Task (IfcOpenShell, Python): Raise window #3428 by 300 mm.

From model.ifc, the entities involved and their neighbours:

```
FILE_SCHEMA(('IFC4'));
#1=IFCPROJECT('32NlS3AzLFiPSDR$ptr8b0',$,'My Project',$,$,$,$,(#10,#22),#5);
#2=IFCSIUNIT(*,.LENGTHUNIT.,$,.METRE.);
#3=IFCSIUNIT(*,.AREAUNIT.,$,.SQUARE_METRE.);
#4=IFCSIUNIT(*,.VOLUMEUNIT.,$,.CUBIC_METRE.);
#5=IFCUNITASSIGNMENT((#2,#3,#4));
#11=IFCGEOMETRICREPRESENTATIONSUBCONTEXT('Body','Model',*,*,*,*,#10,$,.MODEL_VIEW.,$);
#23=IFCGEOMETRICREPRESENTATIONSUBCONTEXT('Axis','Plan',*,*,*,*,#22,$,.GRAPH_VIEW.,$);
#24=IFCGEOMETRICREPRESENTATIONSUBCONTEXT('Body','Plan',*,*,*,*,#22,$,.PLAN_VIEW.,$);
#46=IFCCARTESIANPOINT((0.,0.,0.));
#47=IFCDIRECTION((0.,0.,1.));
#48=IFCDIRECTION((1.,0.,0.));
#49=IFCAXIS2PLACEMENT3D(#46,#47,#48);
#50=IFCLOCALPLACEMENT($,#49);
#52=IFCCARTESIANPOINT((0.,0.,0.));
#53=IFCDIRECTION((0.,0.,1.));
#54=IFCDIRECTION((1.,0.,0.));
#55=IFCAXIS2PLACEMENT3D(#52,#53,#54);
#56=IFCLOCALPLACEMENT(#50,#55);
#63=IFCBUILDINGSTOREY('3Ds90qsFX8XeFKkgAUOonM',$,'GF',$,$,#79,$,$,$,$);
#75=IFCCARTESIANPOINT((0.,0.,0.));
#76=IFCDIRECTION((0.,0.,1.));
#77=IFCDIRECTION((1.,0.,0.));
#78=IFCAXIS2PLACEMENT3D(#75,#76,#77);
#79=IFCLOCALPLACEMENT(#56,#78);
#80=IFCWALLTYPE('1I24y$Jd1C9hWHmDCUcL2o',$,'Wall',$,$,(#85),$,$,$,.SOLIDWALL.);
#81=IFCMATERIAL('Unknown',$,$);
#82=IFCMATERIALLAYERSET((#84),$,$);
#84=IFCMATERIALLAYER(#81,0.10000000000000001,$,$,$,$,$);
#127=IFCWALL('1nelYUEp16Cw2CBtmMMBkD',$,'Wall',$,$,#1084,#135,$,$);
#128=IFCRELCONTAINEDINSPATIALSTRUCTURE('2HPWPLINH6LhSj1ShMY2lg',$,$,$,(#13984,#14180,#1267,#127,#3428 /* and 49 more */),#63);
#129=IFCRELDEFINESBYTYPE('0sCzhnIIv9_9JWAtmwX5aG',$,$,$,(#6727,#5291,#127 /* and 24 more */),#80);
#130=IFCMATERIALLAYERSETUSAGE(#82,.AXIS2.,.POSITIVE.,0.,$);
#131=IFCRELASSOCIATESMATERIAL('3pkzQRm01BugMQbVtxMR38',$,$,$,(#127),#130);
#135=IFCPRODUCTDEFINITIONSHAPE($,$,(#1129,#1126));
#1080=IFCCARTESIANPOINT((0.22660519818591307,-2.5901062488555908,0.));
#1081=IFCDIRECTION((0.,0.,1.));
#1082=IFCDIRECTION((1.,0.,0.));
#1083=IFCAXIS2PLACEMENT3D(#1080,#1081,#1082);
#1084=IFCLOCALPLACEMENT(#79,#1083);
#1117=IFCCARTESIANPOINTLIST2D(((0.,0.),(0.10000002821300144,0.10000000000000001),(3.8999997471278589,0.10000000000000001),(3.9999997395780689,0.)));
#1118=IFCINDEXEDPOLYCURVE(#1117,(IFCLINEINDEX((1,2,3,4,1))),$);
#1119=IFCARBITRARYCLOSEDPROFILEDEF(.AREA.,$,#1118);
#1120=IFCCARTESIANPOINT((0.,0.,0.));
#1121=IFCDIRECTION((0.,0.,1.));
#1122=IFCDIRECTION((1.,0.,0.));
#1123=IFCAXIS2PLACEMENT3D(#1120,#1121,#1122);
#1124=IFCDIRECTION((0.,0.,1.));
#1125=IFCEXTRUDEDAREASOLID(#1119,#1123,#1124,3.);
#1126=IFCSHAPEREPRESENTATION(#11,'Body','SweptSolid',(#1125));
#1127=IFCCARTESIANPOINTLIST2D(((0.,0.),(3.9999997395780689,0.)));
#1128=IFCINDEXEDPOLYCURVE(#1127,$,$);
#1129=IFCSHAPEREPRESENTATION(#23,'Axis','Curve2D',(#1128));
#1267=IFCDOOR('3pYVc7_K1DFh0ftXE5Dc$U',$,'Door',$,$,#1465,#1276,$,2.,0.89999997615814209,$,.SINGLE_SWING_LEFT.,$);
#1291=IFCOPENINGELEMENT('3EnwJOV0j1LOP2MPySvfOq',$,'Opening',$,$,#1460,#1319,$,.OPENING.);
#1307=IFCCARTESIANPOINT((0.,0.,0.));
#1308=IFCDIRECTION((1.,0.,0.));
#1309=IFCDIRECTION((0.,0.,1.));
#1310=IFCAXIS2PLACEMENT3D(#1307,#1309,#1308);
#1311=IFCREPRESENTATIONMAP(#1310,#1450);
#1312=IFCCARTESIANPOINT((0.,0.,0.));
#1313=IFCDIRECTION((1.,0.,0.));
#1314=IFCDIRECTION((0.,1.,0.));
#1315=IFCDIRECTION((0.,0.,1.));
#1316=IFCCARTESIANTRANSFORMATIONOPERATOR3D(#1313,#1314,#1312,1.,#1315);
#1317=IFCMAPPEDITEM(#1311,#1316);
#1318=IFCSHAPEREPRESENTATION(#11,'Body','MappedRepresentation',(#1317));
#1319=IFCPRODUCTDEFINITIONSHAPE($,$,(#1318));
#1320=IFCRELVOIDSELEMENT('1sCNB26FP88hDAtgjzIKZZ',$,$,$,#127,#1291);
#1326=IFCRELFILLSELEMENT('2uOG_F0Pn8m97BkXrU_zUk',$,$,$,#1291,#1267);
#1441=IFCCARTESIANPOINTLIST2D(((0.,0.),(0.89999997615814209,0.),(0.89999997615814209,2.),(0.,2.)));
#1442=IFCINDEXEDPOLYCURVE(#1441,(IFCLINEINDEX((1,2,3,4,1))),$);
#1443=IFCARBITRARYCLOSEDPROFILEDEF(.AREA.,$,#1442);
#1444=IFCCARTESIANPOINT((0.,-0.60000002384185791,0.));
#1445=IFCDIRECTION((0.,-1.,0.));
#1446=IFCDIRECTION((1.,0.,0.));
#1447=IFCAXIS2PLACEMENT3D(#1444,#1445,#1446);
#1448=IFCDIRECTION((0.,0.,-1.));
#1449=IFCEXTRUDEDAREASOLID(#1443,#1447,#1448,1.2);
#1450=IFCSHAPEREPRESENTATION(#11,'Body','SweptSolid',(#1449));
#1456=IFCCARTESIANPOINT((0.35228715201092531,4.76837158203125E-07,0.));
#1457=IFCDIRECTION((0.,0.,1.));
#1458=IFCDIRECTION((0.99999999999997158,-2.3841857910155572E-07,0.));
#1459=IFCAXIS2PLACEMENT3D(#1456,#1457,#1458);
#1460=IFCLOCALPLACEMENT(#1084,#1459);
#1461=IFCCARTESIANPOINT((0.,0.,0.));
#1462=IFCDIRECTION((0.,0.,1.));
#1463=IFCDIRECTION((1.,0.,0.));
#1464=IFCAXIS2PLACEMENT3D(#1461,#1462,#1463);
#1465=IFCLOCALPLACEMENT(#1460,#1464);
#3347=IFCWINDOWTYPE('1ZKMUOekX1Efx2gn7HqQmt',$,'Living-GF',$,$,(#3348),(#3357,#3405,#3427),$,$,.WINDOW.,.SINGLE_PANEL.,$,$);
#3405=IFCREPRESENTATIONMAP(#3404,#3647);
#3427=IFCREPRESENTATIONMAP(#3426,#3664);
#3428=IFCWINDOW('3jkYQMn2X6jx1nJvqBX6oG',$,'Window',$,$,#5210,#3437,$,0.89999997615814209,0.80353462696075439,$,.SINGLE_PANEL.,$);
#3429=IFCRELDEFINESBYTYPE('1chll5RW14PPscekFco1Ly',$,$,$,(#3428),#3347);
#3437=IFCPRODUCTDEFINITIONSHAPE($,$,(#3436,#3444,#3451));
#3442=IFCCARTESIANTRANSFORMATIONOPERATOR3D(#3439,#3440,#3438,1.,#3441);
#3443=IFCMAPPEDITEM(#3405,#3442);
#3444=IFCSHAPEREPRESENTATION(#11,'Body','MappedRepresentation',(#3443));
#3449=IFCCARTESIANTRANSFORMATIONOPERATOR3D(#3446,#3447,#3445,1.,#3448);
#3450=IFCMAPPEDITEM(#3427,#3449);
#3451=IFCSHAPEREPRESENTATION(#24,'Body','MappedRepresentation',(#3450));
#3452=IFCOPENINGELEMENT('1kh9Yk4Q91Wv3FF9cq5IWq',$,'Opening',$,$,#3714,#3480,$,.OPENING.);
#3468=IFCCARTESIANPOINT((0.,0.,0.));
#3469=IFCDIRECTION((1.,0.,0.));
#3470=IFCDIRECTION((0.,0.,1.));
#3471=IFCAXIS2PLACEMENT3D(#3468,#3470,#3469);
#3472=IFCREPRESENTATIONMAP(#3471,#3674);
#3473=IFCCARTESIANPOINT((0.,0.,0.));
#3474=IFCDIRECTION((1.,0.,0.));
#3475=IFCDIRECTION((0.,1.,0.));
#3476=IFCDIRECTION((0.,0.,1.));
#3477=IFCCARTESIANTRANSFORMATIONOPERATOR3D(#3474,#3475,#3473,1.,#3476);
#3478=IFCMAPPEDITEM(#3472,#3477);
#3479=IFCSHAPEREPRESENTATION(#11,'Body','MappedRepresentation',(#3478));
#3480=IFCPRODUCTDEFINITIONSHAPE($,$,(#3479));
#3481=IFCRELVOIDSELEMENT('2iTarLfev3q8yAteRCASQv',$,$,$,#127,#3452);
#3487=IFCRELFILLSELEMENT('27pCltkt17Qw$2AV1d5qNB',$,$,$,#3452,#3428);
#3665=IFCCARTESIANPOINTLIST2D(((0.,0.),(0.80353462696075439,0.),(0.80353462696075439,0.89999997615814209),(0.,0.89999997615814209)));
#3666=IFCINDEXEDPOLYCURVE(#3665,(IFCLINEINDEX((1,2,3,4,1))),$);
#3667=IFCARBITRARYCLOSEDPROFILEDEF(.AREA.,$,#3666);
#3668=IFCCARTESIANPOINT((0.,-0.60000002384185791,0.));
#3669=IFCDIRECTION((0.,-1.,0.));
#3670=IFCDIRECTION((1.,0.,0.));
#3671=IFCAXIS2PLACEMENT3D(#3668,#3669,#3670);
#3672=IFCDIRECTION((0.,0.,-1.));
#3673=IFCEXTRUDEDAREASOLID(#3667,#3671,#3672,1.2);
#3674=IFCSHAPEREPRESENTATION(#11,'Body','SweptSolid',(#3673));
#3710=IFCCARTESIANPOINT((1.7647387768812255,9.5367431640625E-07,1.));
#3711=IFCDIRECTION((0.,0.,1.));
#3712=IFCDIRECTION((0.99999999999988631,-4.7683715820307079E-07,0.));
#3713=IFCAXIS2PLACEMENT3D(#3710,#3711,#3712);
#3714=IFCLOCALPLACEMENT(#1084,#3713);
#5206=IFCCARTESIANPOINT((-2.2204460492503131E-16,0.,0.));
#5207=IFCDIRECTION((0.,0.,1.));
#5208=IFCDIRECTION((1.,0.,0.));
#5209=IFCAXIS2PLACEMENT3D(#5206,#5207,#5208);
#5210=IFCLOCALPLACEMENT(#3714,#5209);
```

```python
import numpy as np
import ifcopenshell
import ifcopenshell.api.geometry
import ifcopenshell.util.placement
import ifcopenshell.util.unit

model = ifcopenshell.open("model.ifc")
unit_scale = ifcopenshell.util.unit.calculate_unit_scale(model)

window = model.by_guid("3jkYQMn2X6jx1nJvqBX6oG")
opening = window.FillsVoids[0].RelatingOpeningElement
dz = 0.3

shift = np.array([0.0, 0.0, dz])
# The window is placed relative to its opening, so it follows when the opening moves.
matrix = ifcopenshell.util.placement.get_local_placement(opening.ObjectPlacement)
matrix[:3, 3] += shift
ifcopenshell.api.geometry.edit_object_placement(
    model, product=opening, matrix=matrix, is_si=False, should_transform_children=True
)

print(f"moved by {dz * unit_scale:+.3f} m")

model.write("model_updated.ifc")
```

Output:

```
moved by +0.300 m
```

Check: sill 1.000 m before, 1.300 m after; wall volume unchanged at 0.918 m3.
